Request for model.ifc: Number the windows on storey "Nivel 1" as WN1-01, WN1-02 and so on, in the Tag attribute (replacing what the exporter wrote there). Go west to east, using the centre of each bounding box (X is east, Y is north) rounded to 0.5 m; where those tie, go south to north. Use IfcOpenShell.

First a look at what the model holds.

```python
import ifcopenshell
import ifcopenshell.util.element
import ifcopenshell.util.placement

model = ifcopenshell.open("model.ifc")
print(model.schema)
storey = next(s for s in model.by_type("IfcBuildingStorey") if s.Name == "Nivel 1")
windows = [e for e in ifcopenshell.util.element.get_decomposition(storey) if e.is_a("IfcWindow")]
for e in sorted(windows, key=lambda e: e.id()):
    origin = ifcopenshell.util.placement.get_local_placement(e.ObjectPlacement)[:3, 3]
    print(e.id(), e.Tag, e.Name, origin.round(2) + 0.0, sep=" | ")
```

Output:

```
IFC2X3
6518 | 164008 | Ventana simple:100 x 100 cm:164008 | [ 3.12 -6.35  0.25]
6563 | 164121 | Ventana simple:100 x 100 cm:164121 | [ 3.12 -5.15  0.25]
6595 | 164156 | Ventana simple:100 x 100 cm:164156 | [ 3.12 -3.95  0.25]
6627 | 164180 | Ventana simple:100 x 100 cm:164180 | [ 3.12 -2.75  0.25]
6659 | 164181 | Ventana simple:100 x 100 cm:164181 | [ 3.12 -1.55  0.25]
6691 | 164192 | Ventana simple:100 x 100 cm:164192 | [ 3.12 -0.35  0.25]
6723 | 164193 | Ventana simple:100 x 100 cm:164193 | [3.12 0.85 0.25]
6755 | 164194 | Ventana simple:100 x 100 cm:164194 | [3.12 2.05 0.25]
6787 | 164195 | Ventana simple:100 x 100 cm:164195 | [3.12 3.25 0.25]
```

```python
import ifcopenshell
import ifcopenshell.geom
import ifcopenshell.util.element
import ifcopenshell.util.shape

model = ifcopenshell.open("model.ifc")
settings = ifcopenshell.geom.settings()
settings.set("use-world-coords", True)


def centre(element):
    shape = ifcopenshell.geom.create_shape(settings, element)
    return ifcopenshell.util.shape.get_bbox_centroid(shape.geometry)


storey = next(s for s in model.by_type("IfcBuildingStorey") if s.Name == "Nivel 1")
windows = [e for e in ifcopenshell.util.element.get_decomposition(storey) if e.is_a("IfcWindow")]

# Insertion points can sit at a corner or the storey origin, so sort by the geometry (in metres).
centres = {e: centre(e) for e in windows}
windows.sort(key=lambda e: (round(centres[e][0] / 0.5), centres[e][1]))

for i, e in enumerate(windows, start=1):
    number = f"WN1-{i:02d}"
    e.Tag = number
    print(e.id(), number)

model.write("model_v2.ifc")
```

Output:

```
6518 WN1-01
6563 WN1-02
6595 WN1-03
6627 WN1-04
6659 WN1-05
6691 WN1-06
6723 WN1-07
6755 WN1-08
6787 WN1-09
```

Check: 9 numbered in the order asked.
